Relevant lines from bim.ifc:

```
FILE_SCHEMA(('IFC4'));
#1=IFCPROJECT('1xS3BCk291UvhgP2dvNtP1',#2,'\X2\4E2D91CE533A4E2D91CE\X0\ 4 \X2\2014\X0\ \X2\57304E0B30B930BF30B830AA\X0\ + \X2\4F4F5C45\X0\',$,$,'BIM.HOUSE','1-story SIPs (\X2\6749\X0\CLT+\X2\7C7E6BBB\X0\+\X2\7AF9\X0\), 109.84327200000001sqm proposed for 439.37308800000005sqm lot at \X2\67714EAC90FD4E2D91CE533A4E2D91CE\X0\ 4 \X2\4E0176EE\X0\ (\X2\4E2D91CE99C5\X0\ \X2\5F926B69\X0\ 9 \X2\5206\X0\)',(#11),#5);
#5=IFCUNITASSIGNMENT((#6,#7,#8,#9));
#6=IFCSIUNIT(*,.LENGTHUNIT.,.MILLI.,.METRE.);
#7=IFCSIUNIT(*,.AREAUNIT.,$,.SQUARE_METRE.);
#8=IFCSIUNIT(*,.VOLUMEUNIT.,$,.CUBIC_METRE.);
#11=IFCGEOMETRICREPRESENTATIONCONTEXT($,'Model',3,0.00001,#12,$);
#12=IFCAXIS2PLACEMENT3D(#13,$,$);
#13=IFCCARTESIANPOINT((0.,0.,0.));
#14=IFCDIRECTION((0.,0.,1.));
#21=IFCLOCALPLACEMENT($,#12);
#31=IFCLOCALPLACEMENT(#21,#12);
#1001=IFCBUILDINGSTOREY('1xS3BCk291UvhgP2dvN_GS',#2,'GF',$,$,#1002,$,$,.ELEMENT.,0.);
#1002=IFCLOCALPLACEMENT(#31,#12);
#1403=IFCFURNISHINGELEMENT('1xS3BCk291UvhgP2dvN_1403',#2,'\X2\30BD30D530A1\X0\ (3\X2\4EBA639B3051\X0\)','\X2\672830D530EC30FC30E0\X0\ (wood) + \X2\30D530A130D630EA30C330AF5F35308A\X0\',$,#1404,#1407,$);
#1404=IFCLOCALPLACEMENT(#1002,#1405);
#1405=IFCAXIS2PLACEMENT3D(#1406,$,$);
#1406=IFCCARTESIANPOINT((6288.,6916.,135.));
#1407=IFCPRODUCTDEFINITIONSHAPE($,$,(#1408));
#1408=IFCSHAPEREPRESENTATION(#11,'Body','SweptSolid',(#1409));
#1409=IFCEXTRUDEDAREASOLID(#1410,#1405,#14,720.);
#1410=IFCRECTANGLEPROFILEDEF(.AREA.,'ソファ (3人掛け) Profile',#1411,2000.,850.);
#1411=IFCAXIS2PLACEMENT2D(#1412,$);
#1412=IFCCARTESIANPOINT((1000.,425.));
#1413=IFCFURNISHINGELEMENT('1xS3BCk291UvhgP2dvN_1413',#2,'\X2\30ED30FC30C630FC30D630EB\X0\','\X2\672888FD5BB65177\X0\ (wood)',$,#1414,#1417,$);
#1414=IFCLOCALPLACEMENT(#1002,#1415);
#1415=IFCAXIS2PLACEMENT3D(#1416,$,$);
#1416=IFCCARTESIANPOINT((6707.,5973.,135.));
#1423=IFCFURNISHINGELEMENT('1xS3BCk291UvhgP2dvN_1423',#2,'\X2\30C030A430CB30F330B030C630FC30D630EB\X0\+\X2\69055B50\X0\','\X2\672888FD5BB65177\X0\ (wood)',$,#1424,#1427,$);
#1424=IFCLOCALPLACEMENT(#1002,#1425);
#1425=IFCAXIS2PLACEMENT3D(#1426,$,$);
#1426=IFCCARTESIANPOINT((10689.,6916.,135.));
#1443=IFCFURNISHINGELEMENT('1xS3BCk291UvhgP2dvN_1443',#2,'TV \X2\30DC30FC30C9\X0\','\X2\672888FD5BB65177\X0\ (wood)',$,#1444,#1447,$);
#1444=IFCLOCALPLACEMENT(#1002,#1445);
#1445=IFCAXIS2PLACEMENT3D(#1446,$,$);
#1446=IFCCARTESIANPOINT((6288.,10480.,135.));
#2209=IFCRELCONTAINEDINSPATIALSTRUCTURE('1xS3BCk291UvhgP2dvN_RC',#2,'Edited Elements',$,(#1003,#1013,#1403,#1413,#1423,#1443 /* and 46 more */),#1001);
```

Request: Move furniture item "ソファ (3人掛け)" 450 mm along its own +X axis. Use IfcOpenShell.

```python
import ifcopenshell
import ifcopenshell.api.geometry
import ifcopenshell.util.placement

model = ifcopenshell.open("bim.ifc")

item = model.by_guid("1xS3BCk291UvhgP2dvN_1403")
matrix = ifcopenshell.util.placement.get_local_placement(item.ObjectPlacement)
matrix[:3, 3] += matrix[:3, 0] * 450.0
ifcopenshell.api.geometry.edit_object_placement(model, product=item, matrix=matrix, is_si=False)

print(ifcopenshell.util.placement.get_local_placement(item.ObjectPlacement).round(3) + 0.0)

model.write("bim_v2.ifc")
```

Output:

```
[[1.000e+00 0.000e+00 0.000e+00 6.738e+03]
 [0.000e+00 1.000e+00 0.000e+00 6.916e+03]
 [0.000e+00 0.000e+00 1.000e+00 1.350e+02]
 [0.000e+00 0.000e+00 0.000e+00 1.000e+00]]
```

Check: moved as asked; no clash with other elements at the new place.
